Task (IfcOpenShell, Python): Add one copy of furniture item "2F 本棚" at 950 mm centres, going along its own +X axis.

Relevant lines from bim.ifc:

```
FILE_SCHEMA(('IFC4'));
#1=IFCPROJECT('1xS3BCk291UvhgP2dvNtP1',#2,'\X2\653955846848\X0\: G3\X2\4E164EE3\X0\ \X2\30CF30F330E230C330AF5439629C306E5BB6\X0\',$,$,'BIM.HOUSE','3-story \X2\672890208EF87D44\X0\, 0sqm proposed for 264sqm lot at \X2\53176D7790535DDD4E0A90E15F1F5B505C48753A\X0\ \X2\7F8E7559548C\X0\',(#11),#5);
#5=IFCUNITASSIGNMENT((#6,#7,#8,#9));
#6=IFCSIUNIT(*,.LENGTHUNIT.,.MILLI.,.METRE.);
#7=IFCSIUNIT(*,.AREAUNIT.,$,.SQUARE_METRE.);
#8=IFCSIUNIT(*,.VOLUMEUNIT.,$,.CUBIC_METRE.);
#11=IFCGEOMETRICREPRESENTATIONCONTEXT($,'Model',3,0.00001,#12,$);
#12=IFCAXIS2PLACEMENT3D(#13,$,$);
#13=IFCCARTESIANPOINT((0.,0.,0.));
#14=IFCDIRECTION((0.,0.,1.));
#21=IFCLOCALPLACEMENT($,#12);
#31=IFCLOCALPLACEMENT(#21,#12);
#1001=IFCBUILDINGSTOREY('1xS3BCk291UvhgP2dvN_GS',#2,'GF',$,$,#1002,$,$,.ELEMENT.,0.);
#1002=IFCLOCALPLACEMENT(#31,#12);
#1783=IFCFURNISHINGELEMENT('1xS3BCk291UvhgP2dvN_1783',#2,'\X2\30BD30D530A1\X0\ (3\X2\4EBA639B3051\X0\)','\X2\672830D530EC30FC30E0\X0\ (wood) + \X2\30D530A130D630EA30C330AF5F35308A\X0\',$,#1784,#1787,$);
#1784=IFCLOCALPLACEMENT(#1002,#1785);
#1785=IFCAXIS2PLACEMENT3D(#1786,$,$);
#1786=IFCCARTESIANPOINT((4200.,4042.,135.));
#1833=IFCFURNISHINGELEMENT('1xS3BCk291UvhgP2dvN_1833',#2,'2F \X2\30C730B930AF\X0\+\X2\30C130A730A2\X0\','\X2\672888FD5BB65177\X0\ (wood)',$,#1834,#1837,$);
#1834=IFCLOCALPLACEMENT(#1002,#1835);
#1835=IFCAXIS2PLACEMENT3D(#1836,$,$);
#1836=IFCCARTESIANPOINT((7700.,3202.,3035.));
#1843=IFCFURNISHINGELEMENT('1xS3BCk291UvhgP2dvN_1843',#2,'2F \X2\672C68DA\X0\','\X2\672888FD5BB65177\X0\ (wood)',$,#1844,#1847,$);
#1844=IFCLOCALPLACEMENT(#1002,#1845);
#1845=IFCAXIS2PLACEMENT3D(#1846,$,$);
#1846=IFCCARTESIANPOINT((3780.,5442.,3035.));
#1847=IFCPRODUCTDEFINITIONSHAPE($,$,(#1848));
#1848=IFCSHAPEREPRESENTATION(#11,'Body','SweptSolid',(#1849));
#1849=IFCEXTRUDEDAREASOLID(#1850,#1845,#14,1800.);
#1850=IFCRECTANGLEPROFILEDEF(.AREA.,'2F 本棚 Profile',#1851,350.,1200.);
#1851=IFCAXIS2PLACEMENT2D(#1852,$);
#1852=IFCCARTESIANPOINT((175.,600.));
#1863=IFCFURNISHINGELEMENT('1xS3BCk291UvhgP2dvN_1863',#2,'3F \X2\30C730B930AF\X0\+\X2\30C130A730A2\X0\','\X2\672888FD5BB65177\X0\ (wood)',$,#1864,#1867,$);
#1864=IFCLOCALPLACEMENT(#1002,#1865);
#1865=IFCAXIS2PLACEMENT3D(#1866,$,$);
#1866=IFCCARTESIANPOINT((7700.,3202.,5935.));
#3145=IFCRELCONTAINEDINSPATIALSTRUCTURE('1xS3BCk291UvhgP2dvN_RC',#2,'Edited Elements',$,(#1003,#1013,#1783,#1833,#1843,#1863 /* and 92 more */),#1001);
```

```python
import ifcopenshell
import ifcopenshell.api.geometry
import ifcopenshell.api.root
import ifcopenshell.util.element
import ifcopenshell.util.placement
import ifcopenshell.util.unit

model = ifcopenshell.open("bim.ifc")
unit_scale = ifcopenshell.util.unit.calculate_unit_scale(model)


def reuse_history(source, copy):
    """copy_class also copies each property set's owner history, people and application; keep the originals."""
    for rel in copy.IsDefinedBy:
        if rel.is_a("IfcRelDefinesByProperties") and (history := rel.RelatingPropertyDefinition.OwnerHistory):
            rel.RelatingPropertyDefinition.OwnerHistory = source.OwnerHistory
            ifcopenshell.util.element.remove_deep2(model, history)


source = model.by_id(1843)
base = ifcopenshell.util.placement.get_local_placement(source.ObjectPlacement)
step = base[:3, 0] * 0.95 / unit_scale

for i in range(1, 2):
    copy = ifcopenshell.api.root.copy_class(model, product=source)
    copy.Representation = ifcopenshell.util.element.copy_deep(
        model, source.Representation, exclude=["IfcGeometricRepresentationContext", "IfcRepresentationMap"]
    )
    reuse_history(source, copy)
    matrix = base.copy()
    matrix[:3, 3] += i * step
    print("added at", matrix[:3, 3].round(3) + 0.0)
    ifcopenshell.api.geometry.edit_object_placement(model, product=copy, matrix=matrix, is_si=False)

model.write("bim_rev.ifc")
```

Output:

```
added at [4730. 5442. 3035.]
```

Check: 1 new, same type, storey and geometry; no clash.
